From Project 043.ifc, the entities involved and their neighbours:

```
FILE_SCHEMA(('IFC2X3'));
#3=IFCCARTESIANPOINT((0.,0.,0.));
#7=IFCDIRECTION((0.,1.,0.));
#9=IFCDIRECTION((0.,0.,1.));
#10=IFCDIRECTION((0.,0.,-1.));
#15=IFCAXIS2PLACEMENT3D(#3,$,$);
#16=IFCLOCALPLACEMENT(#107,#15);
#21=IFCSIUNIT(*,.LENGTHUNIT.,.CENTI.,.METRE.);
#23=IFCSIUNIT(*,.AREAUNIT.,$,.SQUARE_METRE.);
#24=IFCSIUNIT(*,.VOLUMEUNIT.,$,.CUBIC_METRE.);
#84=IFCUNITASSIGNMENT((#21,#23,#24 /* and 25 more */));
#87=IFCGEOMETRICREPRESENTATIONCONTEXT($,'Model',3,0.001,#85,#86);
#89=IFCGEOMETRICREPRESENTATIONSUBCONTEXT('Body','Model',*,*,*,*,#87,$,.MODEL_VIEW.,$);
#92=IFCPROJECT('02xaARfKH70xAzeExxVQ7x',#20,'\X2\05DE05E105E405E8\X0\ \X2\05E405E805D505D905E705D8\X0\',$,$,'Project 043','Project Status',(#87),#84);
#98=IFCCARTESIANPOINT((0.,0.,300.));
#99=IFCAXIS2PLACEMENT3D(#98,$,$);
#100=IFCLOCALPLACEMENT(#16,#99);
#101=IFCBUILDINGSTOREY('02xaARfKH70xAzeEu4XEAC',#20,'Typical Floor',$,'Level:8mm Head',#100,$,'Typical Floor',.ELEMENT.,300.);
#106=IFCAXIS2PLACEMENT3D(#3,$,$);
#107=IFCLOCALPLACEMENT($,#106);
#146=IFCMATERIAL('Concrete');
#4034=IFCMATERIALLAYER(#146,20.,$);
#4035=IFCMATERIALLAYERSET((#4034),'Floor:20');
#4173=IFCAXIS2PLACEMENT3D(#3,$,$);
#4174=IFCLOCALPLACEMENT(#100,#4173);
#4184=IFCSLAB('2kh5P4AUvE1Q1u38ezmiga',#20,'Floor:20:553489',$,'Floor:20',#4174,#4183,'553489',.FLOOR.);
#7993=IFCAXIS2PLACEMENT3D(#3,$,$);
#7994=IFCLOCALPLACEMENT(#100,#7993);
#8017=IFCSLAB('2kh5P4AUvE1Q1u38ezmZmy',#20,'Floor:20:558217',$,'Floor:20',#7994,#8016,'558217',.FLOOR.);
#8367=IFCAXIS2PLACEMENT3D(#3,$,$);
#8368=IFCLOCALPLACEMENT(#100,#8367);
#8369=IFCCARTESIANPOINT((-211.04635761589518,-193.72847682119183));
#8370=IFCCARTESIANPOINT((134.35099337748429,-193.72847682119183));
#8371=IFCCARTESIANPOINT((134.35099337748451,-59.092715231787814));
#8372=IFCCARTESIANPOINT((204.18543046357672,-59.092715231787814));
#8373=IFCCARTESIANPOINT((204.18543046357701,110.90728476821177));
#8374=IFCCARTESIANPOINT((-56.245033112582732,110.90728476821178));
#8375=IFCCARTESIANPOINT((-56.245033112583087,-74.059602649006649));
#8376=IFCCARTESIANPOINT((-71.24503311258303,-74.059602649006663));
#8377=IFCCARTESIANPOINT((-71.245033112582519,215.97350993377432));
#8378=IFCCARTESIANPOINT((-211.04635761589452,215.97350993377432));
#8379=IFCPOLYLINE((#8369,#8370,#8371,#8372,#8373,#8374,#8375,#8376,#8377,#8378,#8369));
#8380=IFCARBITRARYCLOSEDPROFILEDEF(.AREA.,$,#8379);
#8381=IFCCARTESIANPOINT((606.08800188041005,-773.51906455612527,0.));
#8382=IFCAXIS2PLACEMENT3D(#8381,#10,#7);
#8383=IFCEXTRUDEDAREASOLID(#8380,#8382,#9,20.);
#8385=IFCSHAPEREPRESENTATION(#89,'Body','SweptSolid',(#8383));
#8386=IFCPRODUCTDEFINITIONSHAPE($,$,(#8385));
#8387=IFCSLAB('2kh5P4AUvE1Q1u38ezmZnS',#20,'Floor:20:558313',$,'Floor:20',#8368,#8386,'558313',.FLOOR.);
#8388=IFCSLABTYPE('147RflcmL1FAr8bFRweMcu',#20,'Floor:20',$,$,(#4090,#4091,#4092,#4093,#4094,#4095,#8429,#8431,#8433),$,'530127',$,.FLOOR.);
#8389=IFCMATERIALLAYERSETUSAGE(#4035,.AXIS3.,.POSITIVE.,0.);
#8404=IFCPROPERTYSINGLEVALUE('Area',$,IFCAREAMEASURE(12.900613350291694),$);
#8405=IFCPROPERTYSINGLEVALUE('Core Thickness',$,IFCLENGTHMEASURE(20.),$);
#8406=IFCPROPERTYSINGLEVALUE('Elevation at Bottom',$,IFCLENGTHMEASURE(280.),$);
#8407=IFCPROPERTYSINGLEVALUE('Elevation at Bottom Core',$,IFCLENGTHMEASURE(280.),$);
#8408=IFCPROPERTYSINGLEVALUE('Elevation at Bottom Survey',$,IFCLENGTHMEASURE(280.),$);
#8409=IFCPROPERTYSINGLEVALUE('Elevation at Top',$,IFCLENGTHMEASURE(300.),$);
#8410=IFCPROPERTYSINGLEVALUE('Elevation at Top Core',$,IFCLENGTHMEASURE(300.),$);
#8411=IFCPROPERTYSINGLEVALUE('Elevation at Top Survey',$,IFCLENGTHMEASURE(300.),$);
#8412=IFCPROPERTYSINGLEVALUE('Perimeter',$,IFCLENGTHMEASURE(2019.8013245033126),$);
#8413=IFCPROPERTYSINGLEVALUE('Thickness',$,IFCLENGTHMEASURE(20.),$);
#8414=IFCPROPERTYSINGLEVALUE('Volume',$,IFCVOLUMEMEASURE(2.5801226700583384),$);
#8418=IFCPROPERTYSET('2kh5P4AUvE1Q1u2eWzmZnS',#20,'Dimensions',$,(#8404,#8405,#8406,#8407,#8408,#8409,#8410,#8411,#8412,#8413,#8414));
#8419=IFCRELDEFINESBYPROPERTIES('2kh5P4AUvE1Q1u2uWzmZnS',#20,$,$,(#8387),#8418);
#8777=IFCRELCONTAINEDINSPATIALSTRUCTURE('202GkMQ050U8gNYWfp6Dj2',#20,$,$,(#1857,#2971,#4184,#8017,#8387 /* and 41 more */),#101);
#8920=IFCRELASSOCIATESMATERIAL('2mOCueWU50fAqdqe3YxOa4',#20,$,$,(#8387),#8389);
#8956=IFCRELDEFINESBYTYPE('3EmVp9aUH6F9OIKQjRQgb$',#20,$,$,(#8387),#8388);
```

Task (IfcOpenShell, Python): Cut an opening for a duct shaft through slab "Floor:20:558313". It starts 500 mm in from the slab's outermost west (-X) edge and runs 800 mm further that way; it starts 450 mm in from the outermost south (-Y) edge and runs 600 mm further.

```python
import numpy as np
import ifcopenshell
import ifcopenshell.api.feature
import ifcopenshell.api.geometry
import ifcopenshell.api.pset
import ifcopenshell.api.root
import ifcopenshell.geom
import ifcopenshell.util.element
import ifcopenshell.util.placement
import ifcopenshell.util.representation
import ifcopenshell.util.shape
import ifcopenshell.util.unit

model = ifcopenshell.open("Project 043.ifc")
unit_scale = ifcopenshell.util.unit.calculate_unit_scale(model)
area_scale = ifcopenshell.util.unit.calculate_unit_scale(model, "AREAUNIT")
volume_scale = ifcopenshell.util.unit.calculate_unit_scale(model, "VOLUMEUNIT")
settings = ifcopenshell.geom.settings()


def volume(element):
    """Net volume in cubic metres, openings subtracted."""
    shape = ifcopenshell.geom.create_shape(settings, element)
    return ifcopenshell.util.shape.get_volume(shape.geometry)


slab = model.by_id(8387)
before = volume(slab)

# Extent in the slab's own axes, in metres. The edges named are its -X and -Y sides.
slab_shape = ifcopenshell.geom.create_shape(settings, slab)
vertices = ifcopenshell.util.shape.get_vertices(slab_shape.geometry)
x_min, y_min, bottom = vertices.min(axis=0)
top = vertices[:, 2].max()

opening = ifcopenshell.api.root.create_entity(model, ifc_class="IfcOpeningElement", name="Duct shaft opening")
context = ifcopenshell.util.representation.get_context(model, "Model", "Body", "MODEL_VIEW")
width, depth = 0.8, 0.6
outline = [(0.0, 0.0), (width, 0.0), (width, depth), (0.0, depth), (0.0, 0.0)]
# Overshoot both faces by 50 mm so the cut is clean.
shape = ifcopenshell.api.geometry.add_slab_representation(
    model, context=context, depth=top - bottom + 0.1, polyline=outline
)
ifcopenshell.api.geometry.assign_representation(model, product=opening, representation=shape)

matrix = ifcopenshell.util.placement.get_local_placement(slab.ObjectPlacement)
matrix[:, 3] = matrix @ np.append(np.array([x_min + 0.5, y_min + 0.45, bottom - 0.05]) / unit_scale, 1.0)
ifcopenshell.api.geometry.edit_object_placement(model, product=opening, matrix=matrix, is_si=False)
ifcopenshell.api.feature.add_feature(model, feature=opening, element=slab)

after = volume(slab)

# Update the slab's stored quantities.
pset = model.by_id(ifcopenshell.util.element.get_pset(slab, "Dimensions", should_inherit=False)["id"])
ifcopenshell.api.pset.edit_pset(model, pset=pset, properties={
    "Area": model.create_entity("IfcAreaMeasure", after / (top - bottom) / area_scale),
    "Volume": model.create_entity("IfcVolumeMeasure", after / volume_scale),
})

print(f"slab volume {before:.3f} -> {after:.3f} m3")

model.write("Project 043_edited.ifc")
```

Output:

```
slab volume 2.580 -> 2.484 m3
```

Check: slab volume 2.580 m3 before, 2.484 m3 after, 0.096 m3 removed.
